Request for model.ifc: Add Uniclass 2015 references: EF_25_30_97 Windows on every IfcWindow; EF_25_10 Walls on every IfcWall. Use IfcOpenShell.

First a look at what the model holds.

```python
import ifcopenshell

model = ifcopenshell.open("model.ifc")
print(model.schema)
print("classifications:", [c.Name for c in model.by_type("IfcClassification")])
for ifc_class in ("IfcDoor", "IfcRoof", "IfcStair", "IfcWall", "IfcWindow"):
    print(ifc_class, len(model.by_type(ifc_class)))
```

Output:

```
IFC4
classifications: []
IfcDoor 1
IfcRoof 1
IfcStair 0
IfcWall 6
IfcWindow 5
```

```python
import ifcopenshell
import ifcopenshell.api.classification

model = ifcopenshell.open("model.ifc")

system = ifcopenshell.api.classification.add_classification(model, classification="Uniclass 2015")

codes = {
    "IfcWindow": ("EF_25_30_97", "Windows"),
    "IfcWall": ("EF_25_10", "Walls"),
}
for ifc_class, (code, name) in codes.items():
    products = model.by_type(ifc_class)
    ifcopenshell.api.classification.add_reference(
        model, products=products, classification=system, identification=code, name=name
    )
    print(code, len(products))

model.write("model-out.ifc")
```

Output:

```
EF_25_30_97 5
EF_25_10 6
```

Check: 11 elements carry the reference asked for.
